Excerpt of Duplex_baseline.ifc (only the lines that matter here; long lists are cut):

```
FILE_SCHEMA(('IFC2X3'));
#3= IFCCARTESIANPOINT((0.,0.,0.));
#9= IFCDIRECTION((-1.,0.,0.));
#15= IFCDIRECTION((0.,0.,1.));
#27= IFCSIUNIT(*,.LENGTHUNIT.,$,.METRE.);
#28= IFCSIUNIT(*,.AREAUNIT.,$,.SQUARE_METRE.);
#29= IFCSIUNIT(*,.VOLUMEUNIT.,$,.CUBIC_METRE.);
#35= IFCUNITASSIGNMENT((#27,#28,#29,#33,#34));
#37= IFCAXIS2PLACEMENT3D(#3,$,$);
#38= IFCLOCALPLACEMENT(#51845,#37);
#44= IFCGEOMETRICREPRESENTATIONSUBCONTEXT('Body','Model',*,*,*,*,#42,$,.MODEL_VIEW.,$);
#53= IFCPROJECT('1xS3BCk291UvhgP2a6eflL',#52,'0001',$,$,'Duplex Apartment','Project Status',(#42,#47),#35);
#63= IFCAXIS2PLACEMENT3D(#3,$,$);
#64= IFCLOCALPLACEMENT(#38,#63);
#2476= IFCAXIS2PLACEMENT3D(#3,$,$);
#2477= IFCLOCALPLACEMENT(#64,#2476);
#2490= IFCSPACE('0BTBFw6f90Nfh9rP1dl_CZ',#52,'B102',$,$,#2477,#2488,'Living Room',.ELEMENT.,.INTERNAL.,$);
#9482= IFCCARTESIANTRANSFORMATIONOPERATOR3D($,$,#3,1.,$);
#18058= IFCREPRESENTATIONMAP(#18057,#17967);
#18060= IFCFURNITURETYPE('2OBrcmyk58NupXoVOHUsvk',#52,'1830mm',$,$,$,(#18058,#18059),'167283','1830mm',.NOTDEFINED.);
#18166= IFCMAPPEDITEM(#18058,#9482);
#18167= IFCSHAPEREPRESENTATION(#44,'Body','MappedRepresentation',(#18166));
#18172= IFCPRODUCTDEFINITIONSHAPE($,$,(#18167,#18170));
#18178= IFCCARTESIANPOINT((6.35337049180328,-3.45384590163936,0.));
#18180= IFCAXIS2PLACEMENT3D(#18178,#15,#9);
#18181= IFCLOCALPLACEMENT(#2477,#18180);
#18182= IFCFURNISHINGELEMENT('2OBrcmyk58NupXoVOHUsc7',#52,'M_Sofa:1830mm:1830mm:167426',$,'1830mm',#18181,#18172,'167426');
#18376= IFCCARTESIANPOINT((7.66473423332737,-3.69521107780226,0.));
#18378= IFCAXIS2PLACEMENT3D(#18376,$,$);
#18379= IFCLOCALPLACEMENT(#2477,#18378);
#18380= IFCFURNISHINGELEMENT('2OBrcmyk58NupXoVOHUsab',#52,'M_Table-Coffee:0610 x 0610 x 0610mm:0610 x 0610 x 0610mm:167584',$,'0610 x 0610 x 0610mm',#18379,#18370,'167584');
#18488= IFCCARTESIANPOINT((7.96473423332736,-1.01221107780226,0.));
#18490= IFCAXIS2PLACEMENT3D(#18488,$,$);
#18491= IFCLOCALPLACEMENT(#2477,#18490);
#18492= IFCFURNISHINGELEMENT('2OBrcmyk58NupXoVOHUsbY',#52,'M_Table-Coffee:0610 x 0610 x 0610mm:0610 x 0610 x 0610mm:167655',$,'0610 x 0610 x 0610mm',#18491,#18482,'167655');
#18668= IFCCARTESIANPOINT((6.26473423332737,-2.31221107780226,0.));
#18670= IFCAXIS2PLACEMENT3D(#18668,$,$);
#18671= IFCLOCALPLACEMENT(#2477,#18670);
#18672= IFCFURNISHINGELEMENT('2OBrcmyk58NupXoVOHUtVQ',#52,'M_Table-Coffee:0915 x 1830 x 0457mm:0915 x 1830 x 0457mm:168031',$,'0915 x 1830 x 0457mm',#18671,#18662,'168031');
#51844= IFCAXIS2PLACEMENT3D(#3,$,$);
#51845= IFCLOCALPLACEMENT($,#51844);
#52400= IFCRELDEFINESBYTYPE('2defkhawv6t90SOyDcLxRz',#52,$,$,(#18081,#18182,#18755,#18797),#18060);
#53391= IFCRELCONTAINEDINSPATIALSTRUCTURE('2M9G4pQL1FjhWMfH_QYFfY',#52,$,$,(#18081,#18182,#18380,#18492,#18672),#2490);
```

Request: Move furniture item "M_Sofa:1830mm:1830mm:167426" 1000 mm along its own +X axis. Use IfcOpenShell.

```python
import ifcopenshell
import ifcopenshell.api.geometry
import ifcopenshell.util.placement

model = ifcopenshell.open("Duplex_baseline.ifc")

item = model.by_guid("2OBrcmyk58NupXoVOHUsc7")
matrix = ifcopenshell.util.placement.get_local_placement(item.ObjectPlacement)
matrix[:3, 3] += matrix[:3, 0] * 1.0
ifcopenshell.api.geometry.edit_object_placement(model, product=item, matrix=matrix, is_si=False)

print(ifcopenshell.util.placement.get_local_placement(item.ObjectPlacement).round(3) + 0.0)

model.write("Duplex_baseline_rev.ifc")
```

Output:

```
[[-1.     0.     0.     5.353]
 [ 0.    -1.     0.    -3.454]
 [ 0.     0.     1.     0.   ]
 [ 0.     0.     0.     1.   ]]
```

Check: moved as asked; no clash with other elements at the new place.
